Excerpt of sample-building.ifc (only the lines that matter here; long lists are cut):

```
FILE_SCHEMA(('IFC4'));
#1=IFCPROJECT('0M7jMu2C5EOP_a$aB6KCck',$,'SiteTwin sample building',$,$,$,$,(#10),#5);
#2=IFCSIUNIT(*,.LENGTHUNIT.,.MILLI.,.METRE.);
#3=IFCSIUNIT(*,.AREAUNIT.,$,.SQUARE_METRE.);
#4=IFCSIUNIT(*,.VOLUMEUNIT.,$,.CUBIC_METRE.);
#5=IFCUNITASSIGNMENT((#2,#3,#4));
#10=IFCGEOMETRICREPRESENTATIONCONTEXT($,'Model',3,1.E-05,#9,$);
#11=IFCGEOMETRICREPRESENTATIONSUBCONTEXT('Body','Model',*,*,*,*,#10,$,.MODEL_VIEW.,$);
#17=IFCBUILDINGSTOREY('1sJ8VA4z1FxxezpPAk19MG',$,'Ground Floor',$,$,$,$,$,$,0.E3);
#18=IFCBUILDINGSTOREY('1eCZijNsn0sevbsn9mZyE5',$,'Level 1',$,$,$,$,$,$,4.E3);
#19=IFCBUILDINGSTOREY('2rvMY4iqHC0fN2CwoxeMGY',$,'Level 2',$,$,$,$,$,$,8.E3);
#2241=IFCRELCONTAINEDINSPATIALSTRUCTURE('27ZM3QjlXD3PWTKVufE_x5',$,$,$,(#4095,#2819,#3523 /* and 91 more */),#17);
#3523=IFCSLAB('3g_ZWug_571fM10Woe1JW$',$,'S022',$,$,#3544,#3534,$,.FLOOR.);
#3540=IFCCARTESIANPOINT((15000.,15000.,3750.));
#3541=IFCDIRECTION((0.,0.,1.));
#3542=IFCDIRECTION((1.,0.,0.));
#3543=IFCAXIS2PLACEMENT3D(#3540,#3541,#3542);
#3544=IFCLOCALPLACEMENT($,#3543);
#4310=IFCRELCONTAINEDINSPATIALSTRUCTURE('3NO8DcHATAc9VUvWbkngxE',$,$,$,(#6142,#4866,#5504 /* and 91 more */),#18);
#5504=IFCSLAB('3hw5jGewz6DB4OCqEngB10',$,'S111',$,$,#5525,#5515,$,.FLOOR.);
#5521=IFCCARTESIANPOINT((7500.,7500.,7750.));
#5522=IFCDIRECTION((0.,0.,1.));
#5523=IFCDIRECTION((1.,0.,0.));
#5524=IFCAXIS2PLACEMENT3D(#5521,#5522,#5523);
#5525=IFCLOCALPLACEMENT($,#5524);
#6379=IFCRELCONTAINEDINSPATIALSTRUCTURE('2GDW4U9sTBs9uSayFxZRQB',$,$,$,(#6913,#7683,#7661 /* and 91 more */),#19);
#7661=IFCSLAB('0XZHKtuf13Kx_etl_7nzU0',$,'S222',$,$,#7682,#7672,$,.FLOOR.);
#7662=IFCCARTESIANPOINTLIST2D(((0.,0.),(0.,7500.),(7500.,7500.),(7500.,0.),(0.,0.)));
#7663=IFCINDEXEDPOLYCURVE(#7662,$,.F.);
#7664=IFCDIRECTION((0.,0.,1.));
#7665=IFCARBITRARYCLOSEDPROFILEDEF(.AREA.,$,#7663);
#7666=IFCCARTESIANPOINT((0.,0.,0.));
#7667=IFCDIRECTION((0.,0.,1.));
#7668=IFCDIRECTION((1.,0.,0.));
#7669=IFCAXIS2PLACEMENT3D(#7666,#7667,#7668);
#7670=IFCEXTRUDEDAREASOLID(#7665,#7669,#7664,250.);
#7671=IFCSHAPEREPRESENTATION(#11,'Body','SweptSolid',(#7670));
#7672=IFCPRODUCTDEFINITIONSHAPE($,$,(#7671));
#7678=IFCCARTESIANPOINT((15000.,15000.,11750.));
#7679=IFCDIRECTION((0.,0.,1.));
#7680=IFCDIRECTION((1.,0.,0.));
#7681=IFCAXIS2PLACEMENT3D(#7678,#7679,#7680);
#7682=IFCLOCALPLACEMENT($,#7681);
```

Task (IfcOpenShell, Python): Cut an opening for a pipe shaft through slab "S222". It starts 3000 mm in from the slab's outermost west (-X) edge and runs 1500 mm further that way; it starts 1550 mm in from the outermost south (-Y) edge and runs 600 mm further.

```python
import numpy as np
import ifcopenshell
import ifcopenshell.api.feature
import ifcopenshell.api.geometry
import ifcopenshell.api.root
import ifcopenshell.geom
import ifcopenshell.util.placement
import ifcopenshell.util.representation
import ifcopenshell.util.shape
import ifcopenshell.util.unit

model = ifcopenshell.open("sample-building.ifc")
unit_scale = ifcopenshell.util.unit.calculate_unit_scale(model)
settings = ifcopenshell.geom.settings()


def volume(element):
    """Net volume in cubic metres, openings subtracted."""
    shape = ifcopenshell.geom.create_shape(settings, element)
    return ifcopenshell.util.shape.get_volume(shape.geometry)


slab = model.by_guid("0XZHKtuf13Kx_etl_7nzU0")
before = volume(slab)

# Extent in the slab's own axes, in metres. The edges named are its -X and -Y sides.
slab_shape = ifcopenshell.geom.create_shape(settings, slab)
vertices = ifcopenshell.util.shape.get_vertices(slab_shape.geometry)
x_min, y_min, bottom = vertices.min(axis=0)
top = vertices[:, 2].max()

opening = ifcopenshell.api.root.create_entity(model, ifc_class="IfcOpeningElement", name="Pipe shaft opening", predefined_type="OPENING")
context = ifcopenshell.util.representation.get_context(model, "Model", "Body", "MODEL_VIEW")
width, depth = 1.5, 0.6
outline = [(0.0, 0.0), (width, 0.0), (width, depth), (0.0, depth), (0.0, 0.0)]
# Overshoot both faces by 50 mm so the cut is clean.
shape = ifcopenshell.api.geometry.add_slab_representation(
    model, context=context, depth=top - bottom + 0.1, polyline=outline
)
ifcopenshell.api.geometry.assign_representation(model, product=opening, representation=shape)

matrix = ifcopenshell.util.placement.get_local_placement(slab.ObjectPlacement)
matrix[:, 3] = matrix @ np.append(np.array([x_min + 3, y_min + 1.55, bottom - 0.05]) / unit_scale, 1.0)
ifcopenshell.api.geometry.edit_object_placement(model, product=opening, matrix=matrix, is_si=False)
ifcopenshell.api.feature.add_feature(model, feature=opening, element=slab)

after = volume(slab)

print(f"slab volume {before:.3f} -> {after:.3f} m3")

model.write("sample-building_edited.ifc")
```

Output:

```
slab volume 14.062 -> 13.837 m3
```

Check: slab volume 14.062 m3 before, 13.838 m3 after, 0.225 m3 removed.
